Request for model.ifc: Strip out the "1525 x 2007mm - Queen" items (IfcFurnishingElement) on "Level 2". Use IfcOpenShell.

First a look at what the model holds.

```python
import ifcopenshell
import ifcopenshell.util.element

model = ifcopenshell.open("model.ifc")
print(model.schema)
storey = next(s for s in model.by_type("IfcBuildingStorey") if s.Name == "Level 2")
furniture = [e for e in ifcopenshell.util.element.get_decomposition(storey) if e.is_a("IfcFurnishingElement")]
seen = {}
for e in furniture:
    element_type = ifcopenshell.util.element.get_type(e)
    name = element_type.Name if element_type not in (None, e) else None
    seen[name] = seen.get(name, 0) + 1
for name, count in sorted(seen.items(), key=str):
    print(count, "x", name)
```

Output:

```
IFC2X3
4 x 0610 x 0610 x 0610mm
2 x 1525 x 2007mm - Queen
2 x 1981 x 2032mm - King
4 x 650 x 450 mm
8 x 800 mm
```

```python
import ifcopenshell
import ifcopenshell.api.root
import ifcopenshell.util.element

model = ifcopenshell.open("model.ifc")

storey = next(s for s in model.by_type("IfcBuildingStorey") if s.Name == "Level 2")
furniture = [e for e in ifcopenshell.util.element.get_decomposition(storey) if e.is_a("IfcFurnishingElement")]
targets = [e for e in furniture if (t := ifcopenshell.util.element.get_type(e)) not in (None, e) and t.Name == "1525 x 2007mm - Queen"]

for e in targets:
    ifcopenshell.api.root.remove_product(model, product=e)
print(len(targets), "removed")

model.write("model_v2.ifc")
```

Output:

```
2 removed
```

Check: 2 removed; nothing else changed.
